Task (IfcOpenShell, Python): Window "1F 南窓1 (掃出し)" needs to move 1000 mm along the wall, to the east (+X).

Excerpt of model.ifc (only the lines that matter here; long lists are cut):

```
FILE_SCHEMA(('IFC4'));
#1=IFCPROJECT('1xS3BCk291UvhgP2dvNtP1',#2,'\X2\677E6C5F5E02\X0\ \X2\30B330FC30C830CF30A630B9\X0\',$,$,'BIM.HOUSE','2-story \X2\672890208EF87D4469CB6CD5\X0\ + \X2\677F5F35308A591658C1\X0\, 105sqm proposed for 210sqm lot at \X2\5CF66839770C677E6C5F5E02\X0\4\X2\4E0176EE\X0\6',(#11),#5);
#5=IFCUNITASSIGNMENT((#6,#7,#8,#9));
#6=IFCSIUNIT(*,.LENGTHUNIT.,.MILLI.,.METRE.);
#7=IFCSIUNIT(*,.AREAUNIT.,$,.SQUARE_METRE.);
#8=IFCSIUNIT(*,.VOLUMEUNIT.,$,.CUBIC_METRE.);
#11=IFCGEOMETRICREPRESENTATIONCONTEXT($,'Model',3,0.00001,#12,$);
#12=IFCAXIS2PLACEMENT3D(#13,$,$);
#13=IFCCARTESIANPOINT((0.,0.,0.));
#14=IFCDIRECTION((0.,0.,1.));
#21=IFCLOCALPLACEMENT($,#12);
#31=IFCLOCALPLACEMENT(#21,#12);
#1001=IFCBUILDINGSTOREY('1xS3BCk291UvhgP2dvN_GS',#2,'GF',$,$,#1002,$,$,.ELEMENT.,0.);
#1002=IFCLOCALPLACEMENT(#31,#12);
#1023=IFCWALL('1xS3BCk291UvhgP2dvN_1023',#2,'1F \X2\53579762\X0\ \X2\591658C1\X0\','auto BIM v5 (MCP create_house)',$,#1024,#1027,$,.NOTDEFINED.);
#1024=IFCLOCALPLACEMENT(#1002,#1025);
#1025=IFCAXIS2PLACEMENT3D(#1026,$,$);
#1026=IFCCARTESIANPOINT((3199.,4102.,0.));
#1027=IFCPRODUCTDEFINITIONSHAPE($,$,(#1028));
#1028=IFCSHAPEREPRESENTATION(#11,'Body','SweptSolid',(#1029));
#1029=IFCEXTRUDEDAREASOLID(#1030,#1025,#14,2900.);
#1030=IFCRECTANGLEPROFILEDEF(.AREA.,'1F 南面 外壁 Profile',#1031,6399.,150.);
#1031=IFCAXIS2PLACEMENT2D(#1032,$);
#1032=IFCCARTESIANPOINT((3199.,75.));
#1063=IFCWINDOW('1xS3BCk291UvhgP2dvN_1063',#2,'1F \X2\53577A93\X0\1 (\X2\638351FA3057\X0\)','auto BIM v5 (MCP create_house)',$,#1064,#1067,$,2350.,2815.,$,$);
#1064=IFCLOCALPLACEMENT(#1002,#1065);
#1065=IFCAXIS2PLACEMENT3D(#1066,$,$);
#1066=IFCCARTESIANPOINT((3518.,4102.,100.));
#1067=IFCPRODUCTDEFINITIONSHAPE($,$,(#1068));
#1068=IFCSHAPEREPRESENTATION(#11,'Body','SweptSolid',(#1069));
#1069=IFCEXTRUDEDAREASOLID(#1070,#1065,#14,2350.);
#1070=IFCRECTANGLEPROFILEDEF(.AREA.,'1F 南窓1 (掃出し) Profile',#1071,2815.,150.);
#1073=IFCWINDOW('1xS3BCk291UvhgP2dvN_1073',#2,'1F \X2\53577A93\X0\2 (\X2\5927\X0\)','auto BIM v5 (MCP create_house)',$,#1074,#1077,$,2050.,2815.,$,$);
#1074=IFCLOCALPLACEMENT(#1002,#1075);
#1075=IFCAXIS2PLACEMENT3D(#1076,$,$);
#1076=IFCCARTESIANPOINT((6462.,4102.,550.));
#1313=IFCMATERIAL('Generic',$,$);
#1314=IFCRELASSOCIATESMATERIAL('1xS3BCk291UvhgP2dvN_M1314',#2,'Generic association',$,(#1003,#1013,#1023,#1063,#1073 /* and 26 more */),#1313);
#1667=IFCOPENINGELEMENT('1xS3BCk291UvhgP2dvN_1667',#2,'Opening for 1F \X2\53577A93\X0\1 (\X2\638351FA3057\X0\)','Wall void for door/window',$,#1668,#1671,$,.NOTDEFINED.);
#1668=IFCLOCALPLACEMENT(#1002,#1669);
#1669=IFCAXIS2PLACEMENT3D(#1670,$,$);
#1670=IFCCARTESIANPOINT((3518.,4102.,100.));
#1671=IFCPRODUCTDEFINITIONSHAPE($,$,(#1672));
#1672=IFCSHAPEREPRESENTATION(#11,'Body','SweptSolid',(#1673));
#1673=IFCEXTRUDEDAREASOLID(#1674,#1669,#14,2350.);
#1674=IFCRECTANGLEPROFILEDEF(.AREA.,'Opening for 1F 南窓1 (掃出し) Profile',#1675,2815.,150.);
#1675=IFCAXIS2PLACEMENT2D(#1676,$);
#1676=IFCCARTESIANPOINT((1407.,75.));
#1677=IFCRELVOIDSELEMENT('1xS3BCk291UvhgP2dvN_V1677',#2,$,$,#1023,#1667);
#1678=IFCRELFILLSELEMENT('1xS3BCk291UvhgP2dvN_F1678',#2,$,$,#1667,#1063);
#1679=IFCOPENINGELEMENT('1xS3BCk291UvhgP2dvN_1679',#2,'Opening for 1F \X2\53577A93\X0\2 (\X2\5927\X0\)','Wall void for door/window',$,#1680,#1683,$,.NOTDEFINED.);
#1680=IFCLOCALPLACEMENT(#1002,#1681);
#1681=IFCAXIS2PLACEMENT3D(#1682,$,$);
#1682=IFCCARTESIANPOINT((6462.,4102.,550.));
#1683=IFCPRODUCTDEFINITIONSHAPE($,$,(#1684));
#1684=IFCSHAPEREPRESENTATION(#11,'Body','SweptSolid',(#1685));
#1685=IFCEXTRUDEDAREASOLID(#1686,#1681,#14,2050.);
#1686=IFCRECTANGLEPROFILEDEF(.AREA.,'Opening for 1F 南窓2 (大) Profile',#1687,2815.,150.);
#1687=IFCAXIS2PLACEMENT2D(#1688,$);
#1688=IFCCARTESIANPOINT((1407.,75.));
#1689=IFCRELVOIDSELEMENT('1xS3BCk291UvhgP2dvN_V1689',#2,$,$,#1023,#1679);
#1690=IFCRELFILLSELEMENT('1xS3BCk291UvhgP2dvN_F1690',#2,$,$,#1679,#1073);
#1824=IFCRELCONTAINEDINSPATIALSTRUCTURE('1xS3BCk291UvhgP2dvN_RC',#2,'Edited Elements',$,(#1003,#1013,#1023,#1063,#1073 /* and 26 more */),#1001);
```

```python
import ifcopenshell
import ifcopenshell.api.geometry
import ifcopenshell.util.placement
import ifcopenshell.util.unit

model = ifcopenshell.open("model.ifc")
unit_scale = ifcopenshell.util.unit.calculate_unit_scale(model)

window = model.by_id(1063)
opening = window.FillsVoids[0].RelatingOpeningElement
wall = opening.VoidsElements[0].RelatingBuildingElement

wall_matrix = ifcopenshell.util.placement.get_local_placement(wall.ObjectPlacement)
shift = wall_matrix[:3, 0] * 1 / unit_scale
before = ifcopenshell.util.placement.get_local_placement(window.ObjectPlacement)[:3, 3].copy()

# The window is not placed relative to its opening, so move both.
for product in (opening, window):
    matrix = ifcopenshell.util.placement.get_local_placement(product.ObjectPlacement)
    matrix[:3, 3] += shift
    ifcopenshell.api.geometry.edit_object_placement(model, product=product, matrix=matrix, is_si=False)

after = ifcopenshell.util.placement.get_local_placement(window.ObjectPlacement)[:3, 3]
print("window moved by", (after - before).round(3) + 0.0)

model.write("model-out.ifc")
```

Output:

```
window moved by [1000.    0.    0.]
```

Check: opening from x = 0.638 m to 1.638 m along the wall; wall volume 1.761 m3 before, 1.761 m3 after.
